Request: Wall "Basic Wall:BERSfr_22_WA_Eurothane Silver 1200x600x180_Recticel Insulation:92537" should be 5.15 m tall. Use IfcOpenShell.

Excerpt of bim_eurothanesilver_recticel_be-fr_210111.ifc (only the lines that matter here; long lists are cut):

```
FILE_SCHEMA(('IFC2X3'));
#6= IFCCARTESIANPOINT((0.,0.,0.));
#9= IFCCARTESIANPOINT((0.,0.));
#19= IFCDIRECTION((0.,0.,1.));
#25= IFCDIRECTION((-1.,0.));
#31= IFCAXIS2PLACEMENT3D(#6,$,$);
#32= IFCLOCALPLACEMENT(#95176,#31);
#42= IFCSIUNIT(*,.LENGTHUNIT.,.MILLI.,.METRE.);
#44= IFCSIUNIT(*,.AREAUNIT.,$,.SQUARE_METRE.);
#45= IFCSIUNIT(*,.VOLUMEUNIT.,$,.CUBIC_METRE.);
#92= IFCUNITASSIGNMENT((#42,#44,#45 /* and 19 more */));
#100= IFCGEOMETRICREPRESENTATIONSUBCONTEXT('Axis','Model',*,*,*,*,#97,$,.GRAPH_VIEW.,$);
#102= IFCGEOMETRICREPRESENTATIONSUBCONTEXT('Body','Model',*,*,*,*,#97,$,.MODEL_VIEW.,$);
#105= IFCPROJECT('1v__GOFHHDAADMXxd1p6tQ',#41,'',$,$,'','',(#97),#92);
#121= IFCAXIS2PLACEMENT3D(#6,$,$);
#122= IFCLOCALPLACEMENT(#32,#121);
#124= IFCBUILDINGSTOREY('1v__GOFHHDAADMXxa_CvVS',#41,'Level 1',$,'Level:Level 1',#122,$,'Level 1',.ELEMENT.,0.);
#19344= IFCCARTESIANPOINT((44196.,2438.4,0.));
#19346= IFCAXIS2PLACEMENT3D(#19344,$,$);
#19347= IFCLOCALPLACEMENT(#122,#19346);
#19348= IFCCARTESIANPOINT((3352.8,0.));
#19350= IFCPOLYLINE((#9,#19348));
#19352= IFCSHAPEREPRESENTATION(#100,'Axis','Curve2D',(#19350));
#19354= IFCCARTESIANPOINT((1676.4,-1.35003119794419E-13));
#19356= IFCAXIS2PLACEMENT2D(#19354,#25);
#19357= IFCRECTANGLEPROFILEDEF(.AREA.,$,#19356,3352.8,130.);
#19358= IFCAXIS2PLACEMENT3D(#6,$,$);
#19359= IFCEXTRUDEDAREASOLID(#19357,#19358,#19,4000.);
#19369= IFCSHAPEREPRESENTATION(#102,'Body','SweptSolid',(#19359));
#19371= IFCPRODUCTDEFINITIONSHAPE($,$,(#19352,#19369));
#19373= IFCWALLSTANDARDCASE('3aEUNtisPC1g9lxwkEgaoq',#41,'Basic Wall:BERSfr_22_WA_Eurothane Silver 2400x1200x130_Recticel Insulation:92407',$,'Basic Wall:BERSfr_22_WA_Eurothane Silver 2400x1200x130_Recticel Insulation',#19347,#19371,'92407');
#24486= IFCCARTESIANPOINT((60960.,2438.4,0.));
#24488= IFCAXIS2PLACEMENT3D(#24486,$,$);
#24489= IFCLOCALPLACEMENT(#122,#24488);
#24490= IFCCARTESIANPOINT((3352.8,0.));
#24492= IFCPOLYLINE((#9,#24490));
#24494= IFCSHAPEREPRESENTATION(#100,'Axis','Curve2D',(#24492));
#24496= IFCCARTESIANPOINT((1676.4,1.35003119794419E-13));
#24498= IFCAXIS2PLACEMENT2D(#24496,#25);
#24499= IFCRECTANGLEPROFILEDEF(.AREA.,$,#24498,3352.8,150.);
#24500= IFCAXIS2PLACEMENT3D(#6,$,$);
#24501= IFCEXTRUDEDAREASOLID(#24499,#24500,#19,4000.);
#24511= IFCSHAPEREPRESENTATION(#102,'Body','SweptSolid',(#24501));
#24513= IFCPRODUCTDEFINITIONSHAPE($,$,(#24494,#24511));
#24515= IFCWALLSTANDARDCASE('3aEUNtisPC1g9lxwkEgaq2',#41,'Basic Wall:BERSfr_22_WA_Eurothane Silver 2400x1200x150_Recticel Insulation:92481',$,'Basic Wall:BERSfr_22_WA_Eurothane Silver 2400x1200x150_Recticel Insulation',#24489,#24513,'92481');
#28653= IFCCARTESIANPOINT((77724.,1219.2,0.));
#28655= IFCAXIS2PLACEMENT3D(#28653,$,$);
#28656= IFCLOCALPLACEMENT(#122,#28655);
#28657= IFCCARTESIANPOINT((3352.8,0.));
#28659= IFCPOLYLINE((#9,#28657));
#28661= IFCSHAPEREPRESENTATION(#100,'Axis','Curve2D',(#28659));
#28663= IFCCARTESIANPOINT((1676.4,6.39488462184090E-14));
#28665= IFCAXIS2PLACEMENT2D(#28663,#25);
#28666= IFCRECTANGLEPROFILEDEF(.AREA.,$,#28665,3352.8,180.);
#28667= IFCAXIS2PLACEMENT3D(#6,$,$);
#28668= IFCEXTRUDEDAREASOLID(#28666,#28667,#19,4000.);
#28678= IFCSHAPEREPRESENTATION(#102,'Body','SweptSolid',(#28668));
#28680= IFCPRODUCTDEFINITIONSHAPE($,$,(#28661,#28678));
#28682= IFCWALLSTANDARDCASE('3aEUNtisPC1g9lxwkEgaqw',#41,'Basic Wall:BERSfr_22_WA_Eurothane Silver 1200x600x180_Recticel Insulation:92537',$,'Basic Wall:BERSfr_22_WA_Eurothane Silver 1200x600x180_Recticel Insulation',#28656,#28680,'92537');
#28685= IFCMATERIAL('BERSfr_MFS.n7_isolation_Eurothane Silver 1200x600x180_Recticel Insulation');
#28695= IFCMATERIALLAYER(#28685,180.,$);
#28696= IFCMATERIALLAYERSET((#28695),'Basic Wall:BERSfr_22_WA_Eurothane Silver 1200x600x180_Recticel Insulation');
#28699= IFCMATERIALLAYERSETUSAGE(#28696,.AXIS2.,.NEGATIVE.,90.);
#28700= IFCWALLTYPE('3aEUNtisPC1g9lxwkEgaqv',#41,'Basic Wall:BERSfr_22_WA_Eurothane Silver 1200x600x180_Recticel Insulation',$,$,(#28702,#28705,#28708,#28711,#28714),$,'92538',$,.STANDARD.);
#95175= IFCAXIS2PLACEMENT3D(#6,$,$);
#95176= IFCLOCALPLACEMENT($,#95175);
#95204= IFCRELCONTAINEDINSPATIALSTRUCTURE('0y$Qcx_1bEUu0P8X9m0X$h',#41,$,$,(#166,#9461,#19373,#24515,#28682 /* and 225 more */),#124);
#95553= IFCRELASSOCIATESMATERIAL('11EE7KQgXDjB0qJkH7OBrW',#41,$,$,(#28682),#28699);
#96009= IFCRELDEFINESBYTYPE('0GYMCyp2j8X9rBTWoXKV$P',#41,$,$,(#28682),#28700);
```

```python
import ifcopenshell
import ifcopenshell.geom
import ifcopenshell.util.representation
import ifcopenshell.util.shape

model = ifcopenshell.open("bim_eurothanesilver_recticel_be-fr_210111.ifc")
settings = ifcopenshell.geom.settings()


def volume(element):
    """Net volume in cubic metres, openings subtracted."""
    shape = ifcopenshell.geom.create_shape(settings, element)
    return ifcopenshell.util.shape.get_volume(shape.geometry)


wall = model.by_id(28682)
before = volume(wall)

body = ifcopenshell.util.representation.get_representation(wall, "Model", "Body")
solid = body.Items[0]
old_height = solid.Depth
solid.Depth = 5150.0
after = volume(wall)

print(f"height {old_height:g} -> {solid.Depth:g}, volume {before:.3f} -> {after:.3f} m3")

model.write("bim_eurothanesilver_recticel_be-fr_210111-out.ifc")
```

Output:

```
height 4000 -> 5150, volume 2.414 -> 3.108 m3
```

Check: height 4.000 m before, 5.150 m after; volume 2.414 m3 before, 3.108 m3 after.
